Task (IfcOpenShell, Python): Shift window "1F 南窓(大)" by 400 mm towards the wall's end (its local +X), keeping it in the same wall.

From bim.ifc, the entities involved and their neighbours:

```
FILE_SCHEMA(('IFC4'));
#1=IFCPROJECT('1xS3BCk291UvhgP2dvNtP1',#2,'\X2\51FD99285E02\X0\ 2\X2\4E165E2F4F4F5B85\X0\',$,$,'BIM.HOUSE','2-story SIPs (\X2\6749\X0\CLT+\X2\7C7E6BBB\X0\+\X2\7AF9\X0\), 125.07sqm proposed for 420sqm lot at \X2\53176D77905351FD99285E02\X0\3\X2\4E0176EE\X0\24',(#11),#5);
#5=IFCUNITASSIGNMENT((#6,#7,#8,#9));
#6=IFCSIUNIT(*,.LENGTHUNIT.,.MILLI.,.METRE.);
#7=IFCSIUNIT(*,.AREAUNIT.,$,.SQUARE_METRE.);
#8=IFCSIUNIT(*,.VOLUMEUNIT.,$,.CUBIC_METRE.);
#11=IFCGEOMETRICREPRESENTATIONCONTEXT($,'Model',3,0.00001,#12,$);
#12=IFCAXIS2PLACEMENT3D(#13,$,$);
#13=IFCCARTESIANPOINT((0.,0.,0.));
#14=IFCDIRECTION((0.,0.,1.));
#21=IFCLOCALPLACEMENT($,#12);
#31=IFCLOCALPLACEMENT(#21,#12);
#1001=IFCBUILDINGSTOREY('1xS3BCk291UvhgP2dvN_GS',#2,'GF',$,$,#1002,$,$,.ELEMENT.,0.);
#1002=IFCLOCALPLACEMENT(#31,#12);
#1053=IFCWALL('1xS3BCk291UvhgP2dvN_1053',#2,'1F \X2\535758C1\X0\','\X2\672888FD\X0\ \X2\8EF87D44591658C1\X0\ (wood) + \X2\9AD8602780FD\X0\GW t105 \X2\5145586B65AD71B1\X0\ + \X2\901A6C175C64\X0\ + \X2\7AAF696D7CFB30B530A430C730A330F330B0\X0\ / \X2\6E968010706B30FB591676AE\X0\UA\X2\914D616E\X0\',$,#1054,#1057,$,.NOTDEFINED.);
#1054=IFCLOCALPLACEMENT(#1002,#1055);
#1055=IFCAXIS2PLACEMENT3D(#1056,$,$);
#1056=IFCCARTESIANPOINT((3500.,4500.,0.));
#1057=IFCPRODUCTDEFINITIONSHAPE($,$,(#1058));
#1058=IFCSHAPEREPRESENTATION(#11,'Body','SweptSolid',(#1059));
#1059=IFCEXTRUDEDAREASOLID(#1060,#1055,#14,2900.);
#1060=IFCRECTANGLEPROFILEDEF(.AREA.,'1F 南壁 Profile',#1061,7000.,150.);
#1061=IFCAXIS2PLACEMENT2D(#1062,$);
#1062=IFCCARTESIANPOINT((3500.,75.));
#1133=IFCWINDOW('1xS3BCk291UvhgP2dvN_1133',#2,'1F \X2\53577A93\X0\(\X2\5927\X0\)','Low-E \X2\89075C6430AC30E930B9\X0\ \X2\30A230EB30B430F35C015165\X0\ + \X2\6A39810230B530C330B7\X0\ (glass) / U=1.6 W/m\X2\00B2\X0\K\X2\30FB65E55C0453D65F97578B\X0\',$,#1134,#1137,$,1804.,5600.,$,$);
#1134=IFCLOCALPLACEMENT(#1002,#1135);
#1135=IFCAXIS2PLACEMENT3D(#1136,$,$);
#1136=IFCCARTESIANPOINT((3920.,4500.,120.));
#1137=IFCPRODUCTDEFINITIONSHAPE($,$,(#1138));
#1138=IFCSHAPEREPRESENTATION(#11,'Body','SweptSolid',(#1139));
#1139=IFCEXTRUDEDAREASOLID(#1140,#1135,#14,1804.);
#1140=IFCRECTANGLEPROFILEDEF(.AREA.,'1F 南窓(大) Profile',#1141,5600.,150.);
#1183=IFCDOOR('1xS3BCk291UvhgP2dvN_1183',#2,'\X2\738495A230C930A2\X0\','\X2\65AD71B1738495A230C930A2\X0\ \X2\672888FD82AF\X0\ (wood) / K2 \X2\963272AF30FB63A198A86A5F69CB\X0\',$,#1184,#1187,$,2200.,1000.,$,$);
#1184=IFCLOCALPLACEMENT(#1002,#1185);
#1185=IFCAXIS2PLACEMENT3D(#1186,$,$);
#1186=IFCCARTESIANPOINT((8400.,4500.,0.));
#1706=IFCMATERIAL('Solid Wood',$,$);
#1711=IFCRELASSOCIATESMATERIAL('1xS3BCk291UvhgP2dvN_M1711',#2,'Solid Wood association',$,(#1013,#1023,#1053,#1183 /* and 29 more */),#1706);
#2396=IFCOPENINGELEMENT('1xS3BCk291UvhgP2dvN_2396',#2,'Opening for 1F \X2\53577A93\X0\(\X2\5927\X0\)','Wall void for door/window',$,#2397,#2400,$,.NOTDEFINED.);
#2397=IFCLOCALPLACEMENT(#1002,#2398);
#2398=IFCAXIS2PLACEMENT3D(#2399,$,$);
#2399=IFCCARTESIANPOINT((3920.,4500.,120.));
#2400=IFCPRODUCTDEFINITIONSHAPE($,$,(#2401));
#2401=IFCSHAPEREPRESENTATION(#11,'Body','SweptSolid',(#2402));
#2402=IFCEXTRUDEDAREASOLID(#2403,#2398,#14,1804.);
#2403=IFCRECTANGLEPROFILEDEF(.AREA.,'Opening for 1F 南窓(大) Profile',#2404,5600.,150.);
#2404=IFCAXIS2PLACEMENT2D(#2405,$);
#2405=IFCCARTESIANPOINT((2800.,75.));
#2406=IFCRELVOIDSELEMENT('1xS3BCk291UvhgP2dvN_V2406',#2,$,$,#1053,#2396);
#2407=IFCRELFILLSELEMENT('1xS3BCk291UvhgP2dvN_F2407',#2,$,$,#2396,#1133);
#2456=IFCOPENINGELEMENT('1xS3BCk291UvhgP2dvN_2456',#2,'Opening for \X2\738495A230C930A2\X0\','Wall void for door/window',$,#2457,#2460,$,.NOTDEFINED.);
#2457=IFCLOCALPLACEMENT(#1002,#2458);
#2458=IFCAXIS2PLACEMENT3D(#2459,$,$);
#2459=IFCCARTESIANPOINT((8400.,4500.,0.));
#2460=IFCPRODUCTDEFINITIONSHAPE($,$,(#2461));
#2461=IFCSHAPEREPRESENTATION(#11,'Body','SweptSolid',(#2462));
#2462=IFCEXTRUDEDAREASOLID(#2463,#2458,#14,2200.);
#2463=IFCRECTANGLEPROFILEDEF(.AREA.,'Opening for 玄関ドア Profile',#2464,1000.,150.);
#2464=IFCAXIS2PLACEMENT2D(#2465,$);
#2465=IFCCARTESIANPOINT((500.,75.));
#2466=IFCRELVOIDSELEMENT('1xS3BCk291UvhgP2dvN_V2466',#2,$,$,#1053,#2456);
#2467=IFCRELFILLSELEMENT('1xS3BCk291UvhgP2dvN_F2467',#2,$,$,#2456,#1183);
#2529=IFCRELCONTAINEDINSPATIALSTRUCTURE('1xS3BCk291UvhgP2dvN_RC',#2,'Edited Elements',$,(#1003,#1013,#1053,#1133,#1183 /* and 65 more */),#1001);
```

```python
import ifcopenshell
import ifcopenshell.api.geometry
import ifcopenshell.util.placement
import ifcopenshell.util.unit

model = ifcopenshell.open("bim.ifc")
unit_scale = ifcopenshell.util.unit.calculate_unit_scale(model)

window = model.by_guid("1xS3BCk291UvhgP2dvN_1133")
opening = window.FillsVoids[0].RelatingOpeningElement
wall = opening.VoidsElements[0].RelatingBuildingElement

wall_matrix = ifcopenshell.util.placement.get_local_placement(wall.ObjectPlacement)
shift = wall_matrix[:3, 0] * 0.4 / unit_scale
before = ifcopenshell.util.placement.get_local_placement(window.ObjectPlacement)[:3, 3].copy()

# The window is not placed relative to its opening, so move both.
for product in (opening, window):
    matrix = ifcopenshell.util.placement.get_local_placement(product.ObjectPlacement)
    matrix[:3, 3] += shift
    ifcopenshell.api.geometry.edit_object_placement(model, product=product, matrix=matrix, is_si=False)

after = ifcopenshell.util.placement.get_local_placement(window.ObjectPlacement)[:3, 3]
print("window moved by", (after - before).round(3) + 0.0)

model.write("bim_edited.ifc")
```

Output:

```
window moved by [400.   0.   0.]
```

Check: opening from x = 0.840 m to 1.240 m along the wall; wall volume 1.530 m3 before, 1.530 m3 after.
